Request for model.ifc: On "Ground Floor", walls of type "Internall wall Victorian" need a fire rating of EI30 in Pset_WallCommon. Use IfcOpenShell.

First a look at what the model holds.

```python
import ifcopenshell
import ifcopenshell.util.element

model = ifcopenshell.open("model.ifc")
print(model.schema)
storey = next(s for s in model.by_type("IfcBuildingStorey") if s.Name == "Ground Floor")
walls = [e for e in ifcopenshell.util.element.get_decomposition(storey) if e.is_a("IfcWall")]
seen = {}
for e in walls:
    element_type = ifcopenshell.util.element.get_type(e)
    key = (element_type.Name if element_type != e and element_type else None, ifcopenshell.util.element.get_pset(e, "Pset_WallCommon", "FireRating"))
    seen[key] = seen.get(key, 0) + 1
for (name, value), count in sorted(seen.items(), key=str):
    print(count, "x", name, "|", value)
```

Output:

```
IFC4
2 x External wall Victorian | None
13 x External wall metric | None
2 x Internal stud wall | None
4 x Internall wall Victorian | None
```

```python
import ifcopenshell
import ifcopenshell.api.pset
import ifcopenshell.util.element

model = ifcopenshell.open("model.ifc")

storey = next(s for s in model.by_type("IfcBuildingStorey") if s.Name == "Ground Floor")
walls = [e for e in ifcopenshell.util.element.get_decomposition(storey) if e.is_a("IfcWall")]

count = 0
for e in walls:
    element_type = ifcopenshell.util.element.get_type(e)
    if element_type in (None, e) or element_type.Name != "Internall wall Victorian":
        continue
    # add_pset returns the element's existing set when there is one.
    pset = ifcopenshell.api.pset.add_pset(model, product=e, name="Pset_WallCommon")
    ifcopenshell.api.pset.edit_pset(model, pset=pset, properties={"FireRating": "EI30"})
    count += 1

print(count, "walls updated")

model.write("model_v2.ifc")
```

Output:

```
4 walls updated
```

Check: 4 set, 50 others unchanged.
